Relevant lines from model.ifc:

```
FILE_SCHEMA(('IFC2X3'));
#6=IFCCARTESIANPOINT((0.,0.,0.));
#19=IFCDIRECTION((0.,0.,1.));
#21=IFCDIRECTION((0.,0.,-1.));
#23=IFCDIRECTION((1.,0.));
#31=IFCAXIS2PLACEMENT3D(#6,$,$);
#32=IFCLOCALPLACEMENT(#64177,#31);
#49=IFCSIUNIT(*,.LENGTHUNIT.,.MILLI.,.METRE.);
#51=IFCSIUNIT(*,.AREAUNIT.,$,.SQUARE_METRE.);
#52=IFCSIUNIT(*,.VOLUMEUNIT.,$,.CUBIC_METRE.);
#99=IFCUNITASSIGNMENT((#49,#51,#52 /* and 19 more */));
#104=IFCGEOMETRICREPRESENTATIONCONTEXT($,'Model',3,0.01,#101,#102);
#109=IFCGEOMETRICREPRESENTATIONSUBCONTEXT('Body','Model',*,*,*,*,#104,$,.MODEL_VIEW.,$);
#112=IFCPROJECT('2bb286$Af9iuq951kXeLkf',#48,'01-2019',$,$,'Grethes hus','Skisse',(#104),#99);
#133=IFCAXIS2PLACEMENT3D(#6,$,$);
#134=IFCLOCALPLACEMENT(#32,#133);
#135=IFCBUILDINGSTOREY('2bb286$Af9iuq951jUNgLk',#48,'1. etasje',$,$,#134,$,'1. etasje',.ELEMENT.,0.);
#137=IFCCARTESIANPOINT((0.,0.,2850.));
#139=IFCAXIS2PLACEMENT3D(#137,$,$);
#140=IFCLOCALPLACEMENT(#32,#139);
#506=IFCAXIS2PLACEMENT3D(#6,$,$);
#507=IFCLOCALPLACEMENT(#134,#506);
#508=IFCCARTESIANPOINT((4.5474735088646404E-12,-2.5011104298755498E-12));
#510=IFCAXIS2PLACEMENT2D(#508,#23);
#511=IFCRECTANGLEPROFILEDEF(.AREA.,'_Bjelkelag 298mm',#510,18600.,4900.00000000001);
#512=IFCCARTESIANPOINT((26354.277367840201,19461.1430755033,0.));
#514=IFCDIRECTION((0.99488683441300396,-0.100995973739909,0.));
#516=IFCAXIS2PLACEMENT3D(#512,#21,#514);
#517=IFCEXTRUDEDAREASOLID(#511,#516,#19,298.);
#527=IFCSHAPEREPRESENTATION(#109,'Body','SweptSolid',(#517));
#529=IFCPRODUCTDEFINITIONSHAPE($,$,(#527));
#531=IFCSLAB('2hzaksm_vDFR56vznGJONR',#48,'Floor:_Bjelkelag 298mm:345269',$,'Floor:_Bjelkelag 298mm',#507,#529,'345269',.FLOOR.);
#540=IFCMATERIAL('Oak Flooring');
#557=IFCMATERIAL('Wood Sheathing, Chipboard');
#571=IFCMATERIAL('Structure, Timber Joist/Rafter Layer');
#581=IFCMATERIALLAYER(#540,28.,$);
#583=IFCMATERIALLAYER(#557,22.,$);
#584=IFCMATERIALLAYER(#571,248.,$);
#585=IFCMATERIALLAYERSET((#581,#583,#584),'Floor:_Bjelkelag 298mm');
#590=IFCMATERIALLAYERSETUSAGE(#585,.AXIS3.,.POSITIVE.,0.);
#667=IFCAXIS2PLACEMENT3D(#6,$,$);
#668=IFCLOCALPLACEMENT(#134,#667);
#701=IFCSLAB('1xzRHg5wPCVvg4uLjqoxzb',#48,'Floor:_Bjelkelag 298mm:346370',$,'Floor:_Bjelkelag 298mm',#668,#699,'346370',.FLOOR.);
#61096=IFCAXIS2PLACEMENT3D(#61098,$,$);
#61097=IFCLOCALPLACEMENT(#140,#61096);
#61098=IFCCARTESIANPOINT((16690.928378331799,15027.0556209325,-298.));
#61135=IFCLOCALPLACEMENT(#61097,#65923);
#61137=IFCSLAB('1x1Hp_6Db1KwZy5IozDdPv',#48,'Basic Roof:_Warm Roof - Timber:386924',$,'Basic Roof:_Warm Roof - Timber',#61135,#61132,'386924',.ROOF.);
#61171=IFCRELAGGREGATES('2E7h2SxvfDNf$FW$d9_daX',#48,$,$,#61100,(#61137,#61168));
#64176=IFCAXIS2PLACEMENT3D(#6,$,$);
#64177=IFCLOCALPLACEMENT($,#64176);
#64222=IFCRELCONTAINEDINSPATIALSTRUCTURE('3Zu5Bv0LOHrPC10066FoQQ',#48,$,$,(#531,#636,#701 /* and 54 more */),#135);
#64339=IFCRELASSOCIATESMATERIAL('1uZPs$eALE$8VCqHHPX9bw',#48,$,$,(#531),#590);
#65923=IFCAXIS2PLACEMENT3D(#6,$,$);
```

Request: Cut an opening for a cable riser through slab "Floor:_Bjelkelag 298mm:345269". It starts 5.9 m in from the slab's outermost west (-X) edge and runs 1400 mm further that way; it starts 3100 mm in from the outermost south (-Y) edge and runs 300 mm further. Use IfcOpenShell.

```python
import numpy as np
import ifcopenshell
import ifcopenshell.api.feature
import ifcopenshell.api.geometry
import ifcopenshell.api.root
import ifcopenshell.geom
import ifcopenshell.util.placement
import ifcopenshell.util.representation
import ifcopenshell.util.shape
import ifcopenshell.util.unit

model = ifcopenshell.open("model.ifc")
unit_scale = ifcopenshell.util.unit.calculate_unit_scale(model)
settings = ifcopenshell.geom.settings()


def volume(element):
    """Net volume in cubic metres, openings subtracted."""
    shape = ifcopenshell.geom.create_shape(settings, element)
    return ifcopenshell.util.shape.get_volume(shape.geometry)


slab = model.by_guid("2hzaksm_vDFR56vznGJONR")
before = volume(slab)

# Extent in the slab's own axes, in metres. The edges named are its -X and -Y sides.
slab_shape = ifcopenshell.geom.create_shape(settings, slab)
vertices = ifcopenshell.util.shape.get_vertices(slab_shape.geometry)
x_min, y_min, bottom = vertices.min(axis=0)
top = vertices[:, 2].max()

opening = ifcopenshell.api.root.create_entity(model, ifc_class="IfcOpeningElement", name="Cable riser opening")
context = ifcopenshell.util.representation.get_context(model, "Model", "Body", "MODEL_VIEW")
width, depth = 1.4, 0.3
outline = [(0.0, 0.0), (width, 0.0), (width, depth), (0.0, depth), (0.0, 0.0)]
# Overshoot both faces by 50 mm so the cut is clean.
shape = ifcopenshell.api.geometry.add_slab_representation(
    model, context=context, depth=top - bottom + 0.1, polyline=outline
)
ifcopenshell.api.geometry.assign_representation(model, product=opening, representation=shape)

matrix = ifcopenshell.util.placement.get_local_placement(slab.ObjectPlacement)
matrix[:, 3] = matrix @ np.append(np.array([x_min + 5.9, y_min + 3.1, bottom - 0.05]) / unit_scale, 1.0)
ifcopenshell.api.geometry.edit_object_placement(model, product=opening, matrix=matrix, is_si=False)
ifcopenshell.api.feature.add_feature(model, feature=opening, element=slab)

after = volume(slab)

print(f"slab volume {before:.3f} -> {after:.3f} m3")

model.write("model_updated.ifc")
```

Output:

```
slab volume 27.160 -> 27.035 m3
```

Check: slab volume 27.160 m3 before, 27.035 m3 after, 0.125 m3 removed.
